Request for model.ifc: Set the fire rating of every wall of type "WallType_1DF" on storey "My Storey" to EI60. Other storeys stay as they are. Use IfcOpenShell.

First a look at what the model holds.

```python
import ifcopenshell
import ifcopenshell.util.element

model = ifcopenshell.open("model.ifc")
print(model.schema)
storey = next(s for s in model.by_type("IfcBuildingStorey") if s.Name == "My Storey")
walls = [e for e in ifcopenshell.util.element.get_decomposition(storey) if e.is_a("IfcWall")]
seen = {}
for e in walls:
    element_type = ifcopenshell.util.element.get_type(e)
    key = (element_type.Name if element_type != e and element_type else None, ifcopenshell.util.element.get_pset(e, "Pset_WallCommon", "FireRating"))
    seen[key] = seen.get(key, 0) + 1
for (name, value), count in sorted(seen.items(), key=str):
    print(count, "x", name, "|", value)
```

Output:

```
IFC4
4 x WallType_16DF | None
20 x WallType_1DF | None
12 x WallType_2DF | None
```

```python
import ifcopenshell
import ifcopenshell.api.pset
import ifcopenshell.util.element

model = ifcopenshell.open("model.ifc")

storey = next(s for s in model.by_type("IfcBuildingStorey") if s.Name == "My Storey")
walls = [e for e in ifcopenshell.util.element.get_decomposition(storey) if e.is_a("IfcWall")]

count = 0
for e in walls:
    element_type = ifcopenshell.util.element.get_type(e)
    if element_type in (None, e) or element_type.Name != "WallType_1DF":
        continue
    # add_pset returns the element's existing set when there is one.
    pset = ifcopenshell.api.pset.add_pset(model, product=e, name="Pset_WallCommon")
    ifcopenshell.api.pset.edit_pset(model, pset=pset, properties={"FireRating": "EI60"})
    count += 1

print(count, "walls updated")

model.write("model_edited.ifc")
```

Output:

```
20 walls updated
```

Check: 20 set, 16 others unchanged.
